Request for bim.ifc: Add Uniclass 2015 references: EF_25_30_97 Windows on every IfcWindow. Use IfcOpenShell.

First a look at what the model holds.

```python
import ifcopenshell

model = ifcopenshell.open("bim.ifc")
print(model.schema)
print("classifications:", [c.Name for c in model.by_type("IfcClassification")])
for ifc_class in ("IfcDoor", "IfcRoof", "IfcStair", "IfcWall", "IfcWindow"):
    print(ifc_class, len(model.by_type(ifc_class)))
```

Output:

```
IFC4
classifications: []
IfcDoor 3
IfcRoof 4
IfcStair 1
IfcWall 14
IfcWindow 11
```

```python
import ifcopenshell
import ifcopenshell.api.classification

model = ifcopenshell.open("bim.ifc")

system = ifcopenshell.api.classification.add_classification(model, classification="Uniclass 2015")

codes = {
    "IfcWindow": ("EF_25_30_97", "Windows"),
}
for ifc_class, (code, name) in codes.items():
    products = model.by_type(ifc_class)
    ifcopenshell.api.classification.add_reference(
        model, products=products, classification=system, identification=code, name=name
    )
    print(code, len(products))

model.write("bim-out.ifc")
```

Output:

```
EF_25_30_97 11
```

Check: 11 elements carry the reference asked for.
